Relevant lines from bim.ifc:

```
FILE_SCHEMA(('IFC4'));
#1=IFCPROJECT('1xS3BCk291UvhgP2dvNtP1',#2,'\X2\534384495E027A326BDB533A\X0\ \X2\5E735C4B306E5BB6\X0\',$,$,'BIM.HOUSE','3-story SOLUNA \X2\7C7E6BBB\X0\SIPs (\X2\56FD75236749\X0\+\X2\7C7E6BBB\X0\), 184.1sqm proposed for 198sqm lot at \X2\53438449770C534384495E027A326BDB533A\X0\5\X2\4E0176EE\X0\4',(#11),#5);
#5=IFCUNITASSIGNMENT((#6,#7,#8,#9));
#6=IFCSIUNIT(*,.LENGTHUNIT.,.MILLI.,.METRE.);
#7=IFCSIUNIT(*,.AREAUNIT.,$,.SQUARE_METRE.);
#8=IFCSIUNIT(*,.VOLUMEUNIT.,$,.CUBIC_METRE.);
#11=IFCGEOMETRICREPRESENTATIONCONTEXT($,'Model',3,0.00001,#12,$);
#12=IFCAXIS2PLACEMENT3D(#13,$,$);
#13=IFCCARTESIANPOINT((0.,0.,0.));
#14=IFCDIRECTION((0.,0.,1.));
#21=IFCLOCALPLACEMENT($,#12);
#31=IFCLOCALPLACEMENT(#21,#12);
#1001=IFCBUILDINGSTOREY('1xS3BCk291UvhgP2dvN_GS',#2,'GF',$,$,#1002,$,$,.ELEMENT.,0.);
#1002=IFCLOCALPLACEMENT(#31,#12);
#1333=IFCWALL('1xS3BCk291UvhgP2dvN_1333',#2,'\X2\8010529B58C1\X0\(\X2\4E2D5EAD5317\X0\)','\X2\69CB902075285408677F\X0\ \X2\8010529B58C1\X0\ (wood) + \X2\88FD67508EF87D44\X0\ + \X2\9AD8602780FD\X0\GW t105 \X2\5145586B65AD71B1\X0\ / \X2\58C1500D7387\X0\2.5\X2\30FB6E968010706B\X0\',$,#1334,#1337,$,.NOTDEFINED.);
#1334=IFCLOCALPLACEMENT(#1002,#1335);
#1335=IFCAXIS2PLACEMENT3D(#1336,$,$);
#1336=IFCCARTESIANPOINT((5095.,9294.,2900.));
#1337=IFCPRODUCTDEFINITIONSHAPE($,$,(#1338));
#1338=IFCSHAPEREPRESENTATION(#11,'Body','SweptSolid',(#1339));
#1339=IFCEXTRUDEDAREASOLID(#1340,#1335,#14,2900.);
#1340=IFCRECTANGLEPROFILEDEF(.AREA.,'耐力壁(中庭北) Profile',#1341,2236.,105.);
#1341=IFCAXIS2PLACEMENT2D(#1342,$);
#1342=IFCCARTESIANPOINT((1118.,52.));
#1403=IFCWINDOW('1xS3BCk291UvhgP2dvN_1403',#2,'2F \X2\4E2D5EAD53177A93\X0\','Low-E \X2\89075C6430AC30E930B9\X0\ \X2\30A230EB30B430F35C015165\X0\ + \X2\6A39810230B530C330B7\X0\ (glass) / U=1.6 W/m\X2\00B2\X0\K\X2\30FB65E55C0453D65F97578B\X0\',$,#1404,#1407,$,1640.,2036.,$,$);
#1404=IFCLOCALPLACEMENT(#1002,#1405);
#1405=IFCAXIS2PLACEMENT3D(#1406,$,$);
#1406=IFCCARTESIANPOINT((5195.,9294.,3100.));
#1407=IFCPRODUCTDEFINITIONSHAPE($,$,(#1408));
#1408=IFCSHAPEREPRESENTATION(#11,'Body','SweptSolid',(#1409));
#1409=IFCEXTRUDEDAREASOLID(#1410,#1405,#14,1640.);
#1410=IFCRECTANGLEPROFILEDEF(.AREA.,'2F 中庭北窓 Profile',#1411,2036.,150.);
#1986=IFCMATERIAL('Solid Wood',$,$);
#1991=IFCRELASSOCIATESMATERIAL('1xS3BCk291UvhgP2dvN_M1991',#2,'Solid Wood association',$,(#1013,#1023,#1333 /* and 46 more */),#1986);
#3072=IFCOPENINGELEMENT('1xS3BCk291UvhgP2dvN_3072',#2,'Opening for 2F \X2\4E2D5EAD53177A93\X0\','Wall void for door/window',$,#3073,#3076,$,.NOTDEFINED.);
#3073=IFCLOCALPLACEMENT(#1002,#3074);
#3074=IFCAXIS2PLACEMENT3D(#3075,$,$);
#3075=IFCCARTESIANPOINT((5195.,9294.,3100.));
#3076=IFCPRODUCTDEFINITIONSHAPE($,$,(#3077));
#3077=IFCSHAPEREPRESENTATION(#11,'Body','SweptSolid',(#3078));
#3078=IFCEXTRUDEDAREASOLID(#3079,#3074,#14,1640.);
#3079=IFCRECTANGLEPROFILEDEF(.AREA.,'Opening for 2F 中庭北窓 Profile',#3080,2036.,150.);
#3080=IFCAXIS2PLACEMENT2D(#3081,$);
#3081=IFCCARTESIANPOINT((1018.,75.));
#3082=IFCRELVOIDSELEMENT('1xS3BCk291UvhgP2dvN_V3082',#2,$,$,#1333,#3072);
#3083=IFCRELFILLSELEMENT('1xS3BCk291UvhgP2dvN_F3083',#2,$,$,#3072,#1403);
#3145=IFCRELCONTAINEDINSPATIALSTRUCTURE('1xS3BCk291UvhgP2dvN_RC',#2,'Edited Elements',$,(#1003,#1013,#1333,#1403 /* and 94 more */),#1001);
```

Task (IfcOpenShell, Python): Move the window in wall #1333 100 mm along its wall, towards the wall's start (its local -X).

```python
import ifcopenshell
import ifcopenshell.api.geometry
import ifcopenshell.util.placement
import ifcopenshell.util.unit

model = ifcopenshell.open("bim.ifc")
unit_scale = ifcopenshell.util.unit.calculate_unit_scale(model)

window = model.by_guid("1xS3BCk291UvhgP2dvN_1403")
opening = window.FillsVoids[0].RelatingOpeningElement
wall = opening.VoidsElements[0].RelatingBuildingElement

wall_matrix = ifcopenshell.util.placement.get_local_placement(wall.ObjectPlacement)
shift = wall_matrix[:3, 0] * -0.1 / unit_scale
before = ifcopenshell.util.placement.get_local_placement(window.ObjectPlacement)[:3, 3].copy()

# The window is not placed relative to its opening, so move both.
for product in (opening, window):
    matrix = ifcopenshell.util.placement.get_local_placement(product.ObjectPlacement)
    matrix[:3, 3] += shift
    ifcopenshell.api.geometry.edit_object_placement(model, product=product, matrix=matrix, is_si=False)

after = ifcopenshell.util.placement.get_local_placement(window.ObjectPlacement)[:3, 3]
print("window moved by", (after - before).round(3) + 0.0)

model.write("bim_edited.ifc")
```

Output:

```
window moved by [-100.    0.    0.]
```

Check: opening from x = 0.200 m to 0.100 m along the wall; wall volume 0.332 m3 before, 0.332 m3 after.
